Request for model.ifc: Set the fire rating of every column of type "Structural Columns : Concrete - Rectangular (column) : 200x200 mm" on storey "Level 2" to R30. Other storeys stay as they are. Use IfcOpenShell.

First a look at what the model holds.

```python
import ifcopenshell
import ifcopenshell.util.element

model = ifcopenshell.open("model.ifc")
print(model.schema)
storey = next(s for s in model.by_type("IfcBuildingStorey") if s.Name == "Level 2")
columns = [e for e in ifcopenshell.util.element.get_decomposition(storey) if e.is_a("IfcColumn")]
seen = {}
for e in columns:
    element_type = ifcopenshell.util.element.get_type(e)
    key = (element_type.Name if element_type != e and element_type else None, ifcopenshell.util.element.get_pset(e, "Pset_ColumnCommon", "FireRating"))
    seen[key] = seen.get(key, 0) + 1
for (name, value), count in sorted(seen.items(), key=str):
    print(count, "x", name, "|", value)
```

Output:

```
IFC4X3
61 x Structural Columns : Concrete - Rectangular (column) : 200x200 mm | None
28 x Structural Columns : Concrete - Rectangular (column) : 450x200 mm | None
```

```python
import ifcopenshell
import ifcopenshell.api.pset
import ifcopenshell.util.element

model = ifcopenshell.open("model.ifc")

storey = next(s for s in model.by_type("IfcBuildingStorey") if s.Name == "Level 2")
columns = [e for e in ifcopenshell.util.element.get_decomposition(storey) if e.is_a("IfcColumn")]

count = 0
for e in columns:
    element_type = ifcopenshell.util.element.get_type(e)
    if element_type in (None, e) or element_type.Name != "Structural Columns : Concrete - Rectangular (column) : 200x200 mm":
        continue
    # add_pset returns the element's existing set when there is one.
    pset = ifcopenshell.api.pset.add_pset(model, product=e, name="Pset_ColumnCommon")
    ifcopenshell.api.pset.edit_pset(model, pset=pset, properties={"FireRating": "R30"})
    count += 1

print(count, "columns updated")

model.write("model-out.ifc")
```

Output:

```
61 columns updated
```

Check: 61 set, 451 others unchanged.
